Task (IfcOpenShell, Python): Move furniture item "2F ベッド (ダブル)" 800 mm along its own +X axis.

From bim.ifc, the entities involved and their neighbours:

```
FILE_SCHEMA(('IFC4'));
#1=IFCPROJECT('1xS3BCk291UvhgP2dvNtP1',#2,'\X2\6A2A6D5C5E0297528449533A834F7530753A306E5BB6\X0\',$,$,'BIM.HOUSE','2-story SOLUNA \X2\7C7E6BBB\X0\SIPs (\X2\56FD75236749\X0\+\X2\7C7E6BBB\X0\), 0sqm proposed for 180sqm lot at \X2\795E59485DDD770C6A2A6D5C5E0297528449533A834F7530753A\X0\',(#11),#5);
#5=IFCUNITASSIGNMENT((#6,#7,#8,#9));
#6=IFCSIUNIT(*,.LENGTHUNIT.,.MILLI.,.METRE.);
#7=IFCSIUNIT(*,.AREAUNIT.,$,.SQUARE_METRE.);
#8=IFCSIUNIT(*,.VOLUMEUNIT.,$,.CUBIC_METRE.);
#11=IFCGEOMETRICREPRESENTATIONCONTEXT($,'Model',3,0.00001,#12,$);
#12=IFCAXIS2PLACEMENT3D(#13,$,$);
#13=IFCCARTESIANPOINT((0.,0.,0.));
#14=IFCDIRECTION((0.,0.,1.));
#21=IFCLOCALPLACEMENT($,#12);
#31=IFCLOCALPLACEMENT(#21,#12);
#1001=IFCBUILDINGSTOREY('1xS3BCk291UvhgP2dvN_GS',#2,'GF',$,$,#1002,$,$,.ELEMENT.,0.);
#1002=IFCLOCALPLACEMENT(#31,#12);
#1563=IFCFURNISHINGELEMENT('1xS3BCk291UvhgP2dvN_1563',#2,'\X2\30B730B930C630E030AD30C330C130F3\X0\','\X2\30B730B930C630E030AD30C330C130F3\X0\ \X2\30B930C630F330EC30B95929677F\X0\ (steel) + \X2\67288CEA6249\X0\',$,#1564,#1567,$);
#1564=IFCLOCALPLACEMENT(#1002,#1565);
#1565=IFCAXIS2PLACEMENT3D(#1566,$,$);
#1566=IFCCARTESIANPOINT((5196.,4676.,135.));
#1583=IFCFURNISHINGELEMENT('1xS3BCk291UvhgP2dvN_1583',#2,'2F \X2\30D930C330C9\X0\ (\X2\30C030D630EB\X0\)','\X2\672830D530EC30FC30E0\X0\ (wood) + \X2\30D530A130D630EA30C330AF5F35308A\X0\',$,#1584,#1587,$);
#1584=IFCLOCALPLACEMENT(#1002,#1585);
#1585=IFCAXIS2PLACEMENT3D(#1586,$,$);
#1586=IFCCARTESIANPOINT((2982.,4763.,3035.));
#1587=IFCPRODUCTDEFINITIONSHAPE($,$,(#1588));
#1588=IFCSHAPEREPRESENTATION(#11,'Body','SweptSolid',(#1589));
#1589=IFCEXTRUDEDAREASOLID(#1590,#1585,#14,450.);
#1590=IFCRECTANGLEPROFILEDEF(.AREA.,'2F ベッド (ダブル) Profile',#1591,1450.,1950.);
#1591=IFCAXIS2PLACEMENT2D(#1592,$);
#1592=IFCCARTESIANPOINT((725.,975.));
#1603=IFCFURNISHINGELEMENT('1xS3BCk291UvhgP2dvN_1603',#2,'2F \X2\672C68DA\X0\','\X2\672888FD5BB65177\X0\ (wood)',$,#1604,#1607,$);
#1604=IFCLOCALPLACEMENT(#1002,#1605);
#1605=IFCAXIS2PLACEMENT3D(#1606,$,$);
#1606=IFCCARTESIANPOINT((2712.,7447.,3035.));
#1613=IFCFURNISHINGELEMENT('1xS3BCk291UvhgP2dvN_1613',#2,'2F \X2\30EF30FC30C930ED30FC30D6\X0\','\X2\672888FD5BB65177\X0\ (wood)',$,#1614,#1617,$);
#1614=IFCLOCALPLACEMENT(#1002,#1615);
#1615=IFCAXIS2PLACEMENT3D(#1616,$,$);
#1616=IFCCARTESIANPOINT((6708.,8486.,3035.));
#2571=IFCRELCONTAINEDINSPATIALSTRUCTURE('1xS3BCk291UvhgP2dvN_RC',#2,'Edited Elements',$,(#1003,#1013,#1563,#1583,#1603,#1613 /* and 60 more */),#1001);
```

```python
import ifcopenshell
import ifcopenshell.api.geometry
import ifcopenshell.util.placement
import ifcopenshell.util.unit

model = ifcopenshell.open("bim.ifc")
unit_scale = ifcopenshell.util.unit.calculate_unit_scale(model)

item = model.by_guid("1xS3BCk291UvhgP2dvN_1583")
matrix = ifcopenshell.util.placement.get_local_placement(item.ObjectPlacement)
matrix[:3, 3] += matrix[:3, 0] * 0.8 / unit_scale
ifcopenshell.api.geometry.edit_object_placement(model, product=item, matrix=matrix, is_si=False)

print(ifcopenshell.util.placement.get_local_placement(item.ObjectPlacement).round(3) + 0.0)

model.write("bim_rev.ifc")
```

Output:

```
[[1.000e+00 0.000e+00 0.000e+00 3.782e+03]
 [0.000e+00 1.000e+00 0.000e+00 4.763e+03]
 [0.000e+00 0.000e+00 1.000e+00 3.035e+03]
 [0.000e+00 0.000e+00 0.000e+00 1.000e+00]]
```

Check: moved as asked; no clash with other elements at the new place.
